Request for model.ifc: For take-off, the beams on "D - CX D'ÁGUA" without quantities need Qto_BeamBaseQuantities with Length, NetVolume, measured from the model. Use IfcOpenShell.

First a look at what the model holds.

```python
import ifcopenshell
import ifcopenshell.util.element
import ifcopenshell.util.unit

model = ifcopenshell.open("model.ifc")
print(model.schema)
for unit_type in ("LENGTHUNIT", "AREAUNIT", "VOLUMEUNIT"):
    print(unit_type, ifcopenshell.util.unit.calculate_unit_scale(model, unit_type))
storey = next(s for s in model.by_type("IfcBuildingStorey") if s.Name == "D - CX D'ÁGUA")
beams = [e for e in ifcopenshell.util.element.get_decomposition(storey) if e.is_a("IfcBeam")]
for e in sorted(beams, key=lambda e: e.id()):
    print(e.id(), e.is_a(), e.Name, list(ifcopenshell.util.element.get_psets(e, qtos_only=True)), sep=" | ")
```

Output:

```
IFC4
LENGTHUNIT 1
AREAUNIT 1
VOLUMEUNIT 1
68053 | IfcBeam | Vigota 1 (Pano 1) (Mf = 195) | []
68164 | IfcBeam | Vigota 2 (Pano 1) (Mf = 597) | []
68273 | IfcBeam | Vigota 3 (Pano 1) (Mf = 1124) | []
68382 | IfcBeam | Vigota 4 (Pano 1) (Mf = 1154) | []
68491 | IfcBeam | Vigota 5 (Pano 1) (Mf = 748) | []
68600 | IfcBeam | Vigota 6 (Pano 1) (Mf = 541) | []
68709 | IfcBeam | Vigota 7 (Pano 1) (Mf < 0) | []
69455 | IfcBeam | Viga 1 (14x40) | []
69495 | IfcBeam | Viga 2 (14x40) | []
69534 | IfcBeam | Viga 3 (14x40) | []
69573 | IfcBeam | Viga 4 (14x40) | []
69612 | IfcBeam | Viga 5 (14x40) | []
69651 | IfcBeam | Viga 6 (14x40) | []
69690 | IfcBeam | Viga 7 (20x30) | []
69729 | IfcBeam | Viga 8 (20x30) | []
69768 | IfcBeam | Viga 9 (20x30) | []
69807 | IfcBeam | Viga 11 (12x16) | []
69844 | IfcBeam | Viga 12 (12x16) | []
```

```python
import ifcopenshell
import ifcopenshell.api.pset
import ifcopenshell.geom
import ifcopenshell.util.element
import ifcopenshell.util.shape
import ifcopenshell.util.unit

model = ifcopenshell.open("model.ifc")
unit_scale = ifcopenshell.util.unit.calculate_unit_scale(model)
volume_scale = ifcopenshell.util.unit.calculate_unit_scale(model, "VOLUMEUNIT")
settings = ifcopenshell.geom.settings()

storey = next(s for s in model.by_type("IfcBuildingStorey") if s.Name == "D - CX D'ÁGUA")
beams = [e for e in ifcopenshell.util.element.get_decomposition(storey) if e.is_a("IfcBeam")]

for e in sorted(beams, key=lambda e: e.id()):
    if ifcopenshell.util.element.get_psets(e, qtos_only=True, should_inherit=False):
        continue
    # Geometry comes back in metres, in the element's own axes.
    shape = ifcopenshell.geom.create_shape(settings, e)
    values = {
        "Length": ifcopenshell.util.shape.get_max_xyz(shape.geometry) / unit_scale,
        "NetVolume": ifcopenshell.util.shape.get_volume(shape.geometry) / volume_scale,
    }
    qto = ifcopenshell.api.pset.add_qto(model, product=e, name="Qto_BeamBaseQuantities")
    ifcopenshell.api.pset.edit_qto(model, qto=qto, properties=values)
    print(e.id(), {k: round(v, 3) for k, v in values.items()})

model.write("model_updated.ifc")
```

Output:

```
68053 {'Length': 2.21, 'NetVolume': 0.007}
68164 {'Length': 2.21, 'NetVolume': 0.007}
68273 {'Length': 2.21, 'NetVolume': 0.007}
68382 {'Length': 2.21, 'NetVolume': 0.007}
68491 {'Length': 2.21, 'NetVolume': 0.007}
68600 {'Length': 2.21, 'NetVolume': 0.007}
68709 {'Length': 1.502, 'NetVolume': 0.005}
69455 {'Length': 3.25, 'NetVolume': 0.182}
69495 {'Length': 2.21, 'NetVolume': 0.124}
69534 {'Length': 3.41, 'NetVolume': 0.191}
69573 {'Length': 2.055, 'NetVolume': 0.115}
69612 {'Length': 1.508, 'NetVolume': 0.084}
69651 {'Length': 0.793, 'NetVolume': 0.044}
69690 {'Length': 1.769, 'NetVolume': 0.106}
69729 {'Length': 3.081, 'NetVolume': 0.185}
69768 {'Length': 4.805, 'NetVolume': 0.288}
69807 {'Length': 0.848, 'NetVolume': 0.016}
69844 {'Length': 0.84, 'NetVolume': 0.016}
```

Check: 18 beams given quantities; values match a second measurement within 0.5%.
